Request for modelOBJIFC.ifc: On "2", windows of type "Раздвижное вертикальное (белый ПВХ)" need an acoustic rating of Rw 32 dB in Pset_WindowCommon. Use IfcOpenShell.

First a look at what the model holds.

```python
import ifcopenshell
import ifcopenshell.util.element

model = ifcopenshell.open("modelOBJIFC.ifc")
print(model.schema)
storey = next(s for s in model.by_type("IfcBuildingStorey") if s.Name == "2")
windows = [e for e in ifcopenshell.util.element.get_decomposition(storey) if e.is_a("IfcWindow")]
seen = {}
for e in windows:
    element_type = ifcopenshell.util.element.get_type(e)
    key = (element_type.Name if element_type != e and element_type else None, ifcopenshell.util.element.get_pset(e, "Pset_WindowCommon", "AcousticRating"))
    seen[key] = seen.get(key, 0) + 1
for (name, value), count in sorted(seen.items(), key=str):
    print(count, "x", name, "|", value)
```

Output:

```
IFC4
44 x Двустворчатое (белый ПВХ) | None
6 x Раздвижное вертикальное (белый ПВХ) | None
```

```python
import ifcopenshell
import ifcopenshell.api.pset
import ifcopenshell.util.element

model = ifcopenshell.open("modelOBJIFC.ifc")

storey = next(s for s in model.by_type("IfcBuildingStorey") if s.Name == "2")
windows = [e for e in ifcopenshell.util.element.get_decomposition(storey) if e.is_a("IfcWindow")]

count = 0
for e in windows:
    element_type = ifcopenshell.util.element.get_type(e)
    if element_type in (None, e) or element_type.Name != "Раздвижное вертикальное (белый ПВХ)":
        continue
    # add_pset returns the element's existing set when there is one.
    pset = ifcopenshell.api.pset.add_pset(model, product=e, name="Pset_WindowCommon")
    ifcopenshell.api.pset.edit_pset(model, pset=pset, properties={"AcousticRating": "Rw 32 dB"})
    count += 1

print(count, "windows updated")

model.write("modelOBJIFC_updated.ifc")
```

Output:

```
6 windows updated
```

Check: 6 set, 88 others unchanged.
